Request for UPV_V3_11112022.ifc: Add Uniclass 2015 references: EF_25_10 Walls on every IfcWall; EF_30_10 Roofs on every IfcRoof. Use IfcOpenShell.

First a look at what the model holds.

```python
import ifcopenshell

model = ifcopenshell.open("UPV_V3_11112022.ifc")
print(model.schema)
print("classifications:", [c.Name for c in model.by_type("IfcClassification")])
for ifc_class in ("IfcDoor", "IfcRoof", "IfcStair", "IfcWall", "IfcWindow"):
    print(ifc_class, len(model.by_type(ifc_class)))
```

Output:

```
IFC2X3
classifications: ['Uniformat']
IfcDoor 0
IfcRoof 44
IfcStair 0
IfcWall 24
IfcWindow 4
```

```python
import ifcopenshell
import ifcopenshell.api.classification

model = ifcopenshell.open("UPV_V3_11112022.ifc")

# IFC2X3 requires Source and Edition and has no link from the project to the system.
system = model.create_entity("IfcClassification", Source="NBS", Edition="2015", Name="Uniclass 2015")

codes = {
    "IfcWall": ("EF_25_10", "Walls"),
    "IfcRoof": ("EF_30_10", "Roofs"),
}
for ifc_class, (code, name) in codes.items():
    products = model.by_type(ifc_class)
    ifcopenshell.api.classification.add_reference(
        model, products=products, classification=system, identification=code, name=name
    )
    print(code, len(products))

model.write("UPV_V3_11112022_v2.ifc")
```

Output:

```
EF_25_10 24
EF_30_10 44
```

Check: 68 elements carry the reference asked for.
